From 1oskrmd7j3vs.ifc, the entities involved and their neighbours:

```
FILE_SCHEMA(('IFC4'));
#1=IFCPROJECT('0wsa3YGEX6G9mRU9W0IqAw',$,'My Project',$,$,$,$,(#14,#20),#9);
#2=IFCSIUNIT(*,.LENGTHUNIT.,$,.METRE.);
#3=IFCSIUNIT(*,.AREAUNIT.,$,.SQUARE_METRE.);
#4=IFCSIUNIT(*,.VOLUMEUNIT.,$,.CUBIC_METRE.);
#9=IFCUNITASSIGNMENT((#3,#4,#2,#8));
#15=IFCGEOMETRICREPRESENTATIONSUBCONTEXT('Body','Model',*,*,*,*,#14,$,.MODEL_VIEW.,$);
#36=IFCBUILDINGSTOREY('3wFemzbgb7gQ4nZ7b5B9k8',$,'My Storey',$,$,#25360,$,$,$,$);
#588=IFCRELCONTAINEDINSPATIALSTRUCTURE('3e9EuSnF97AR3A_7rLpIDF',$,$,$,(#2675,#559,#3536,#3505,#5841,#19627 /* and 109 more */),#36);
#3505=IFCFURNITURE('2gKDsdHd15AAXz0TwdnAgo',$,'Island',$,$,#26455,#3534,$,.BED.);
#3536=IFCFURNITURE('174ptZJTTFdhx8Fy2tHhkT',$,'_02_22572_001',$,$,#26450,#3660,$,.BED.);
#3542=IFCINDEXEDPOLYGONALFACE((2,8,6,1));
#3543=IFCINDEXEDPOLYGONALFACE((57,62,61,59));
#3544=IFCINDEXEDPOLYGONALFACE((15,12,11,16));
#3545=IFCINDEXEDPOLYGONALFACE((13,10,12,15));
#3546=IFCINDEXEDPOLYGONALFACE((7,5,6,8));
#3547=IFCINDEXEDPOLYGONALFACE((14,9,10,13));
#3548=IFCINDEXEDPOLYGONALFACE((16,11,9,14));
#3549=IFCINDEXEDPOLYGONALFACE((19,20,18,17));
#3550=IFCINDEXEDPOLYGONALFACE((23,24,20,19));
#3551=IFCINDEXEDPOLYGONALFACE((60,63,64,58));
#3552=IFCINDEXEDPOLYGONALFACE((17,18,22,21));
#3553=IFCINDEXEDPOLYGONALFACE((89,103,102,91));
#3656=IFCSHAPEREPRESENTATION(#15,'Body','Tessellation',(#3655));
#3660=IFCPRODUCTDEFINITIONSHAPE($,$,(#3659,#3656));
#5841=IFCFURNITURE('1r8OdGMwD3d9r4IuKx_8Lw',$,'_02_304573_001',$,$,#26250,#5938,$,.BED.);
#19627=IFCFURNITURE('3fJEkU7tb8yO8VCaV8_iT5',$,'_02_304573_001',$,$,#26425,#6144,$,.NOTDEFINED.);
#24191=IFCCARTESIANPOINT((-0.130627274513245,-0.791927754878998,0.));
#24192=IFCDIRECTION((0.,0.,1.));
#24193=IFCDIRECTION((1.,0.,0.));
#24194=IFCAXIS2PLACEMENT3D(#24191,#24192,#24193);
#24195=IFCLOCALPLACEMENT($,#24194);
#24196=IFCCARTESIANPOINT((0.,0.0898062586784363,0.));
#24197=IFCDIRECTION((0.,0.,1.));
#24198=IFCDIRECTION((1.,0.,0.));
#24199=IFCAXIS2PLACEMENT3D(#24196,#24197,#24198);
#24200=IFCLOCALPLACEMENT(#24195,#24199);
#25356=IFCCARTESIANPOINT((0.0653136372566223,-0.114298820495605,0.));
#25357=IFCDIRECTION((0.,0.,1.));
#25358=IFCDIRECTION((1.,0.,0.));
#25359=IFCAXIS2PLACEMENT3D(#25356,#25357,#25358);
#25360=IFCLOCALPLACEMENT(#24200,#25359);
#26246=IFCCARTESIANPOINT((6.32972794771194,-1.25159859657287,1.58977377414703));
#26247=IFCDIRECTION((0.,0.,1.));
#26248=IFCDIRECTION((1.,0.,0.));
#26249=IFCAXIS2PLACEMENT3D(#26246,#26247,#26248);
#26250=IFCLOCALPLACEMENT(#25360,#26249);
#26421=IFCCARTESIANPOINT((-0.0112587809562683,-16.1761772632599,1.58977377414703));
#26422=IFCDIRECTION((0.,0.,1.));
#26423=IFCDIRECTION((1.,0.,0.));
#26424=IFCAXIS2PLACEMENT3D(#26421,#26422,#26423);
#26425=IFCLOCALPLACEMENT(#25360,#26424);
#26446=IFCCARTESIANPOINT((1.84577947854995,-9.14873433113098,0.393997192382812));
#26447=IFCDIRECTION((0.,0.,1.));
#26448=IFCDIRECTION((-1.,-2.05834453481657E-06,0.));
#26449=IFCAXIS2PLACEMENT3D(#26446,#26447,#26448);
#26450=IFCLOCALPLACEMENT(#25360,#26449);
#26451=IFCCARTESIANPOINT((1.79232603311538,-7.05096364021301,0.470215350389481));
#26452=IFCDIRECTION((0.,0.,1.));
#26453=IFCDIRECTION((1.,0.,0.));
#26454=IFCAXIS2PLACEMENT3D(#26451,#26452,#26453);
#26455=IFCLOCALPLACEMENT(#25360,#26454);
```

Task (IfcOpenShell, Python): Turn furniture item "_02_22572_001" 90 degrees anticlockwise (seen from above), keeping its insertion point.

```python
import ifcopenshell
import ifcopenshell.api.geometry
import ifcopenshell.util.placement

model = ifcopenshell.open("1oskrmd7j3vs.ifc")

item = model.by_guid("174ptZJTTFdhx8Fy2tHhkT")
matrix = ifcopenshell.util.placement.get_local_placement(item.ObjectPlacement)
matrix = matrix @ ifcopenshell.util.placement.rotation(90, "Z")
ifcopenshell.api.geometry.edit_object_placement(model, product=item, matrix=matrix, is_si=False)

print(ifcopenshell.util.placement.get_local_placement(item.ObjectPlacement).round(3) + 0.0)

model.write("1oskrmd7j3vs_v2.ifc")
```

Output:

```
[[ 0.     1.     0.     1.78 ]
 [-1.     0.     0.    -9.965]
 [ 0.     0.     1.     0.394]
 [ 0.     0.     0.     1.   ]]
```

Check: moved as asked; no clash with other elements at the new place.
